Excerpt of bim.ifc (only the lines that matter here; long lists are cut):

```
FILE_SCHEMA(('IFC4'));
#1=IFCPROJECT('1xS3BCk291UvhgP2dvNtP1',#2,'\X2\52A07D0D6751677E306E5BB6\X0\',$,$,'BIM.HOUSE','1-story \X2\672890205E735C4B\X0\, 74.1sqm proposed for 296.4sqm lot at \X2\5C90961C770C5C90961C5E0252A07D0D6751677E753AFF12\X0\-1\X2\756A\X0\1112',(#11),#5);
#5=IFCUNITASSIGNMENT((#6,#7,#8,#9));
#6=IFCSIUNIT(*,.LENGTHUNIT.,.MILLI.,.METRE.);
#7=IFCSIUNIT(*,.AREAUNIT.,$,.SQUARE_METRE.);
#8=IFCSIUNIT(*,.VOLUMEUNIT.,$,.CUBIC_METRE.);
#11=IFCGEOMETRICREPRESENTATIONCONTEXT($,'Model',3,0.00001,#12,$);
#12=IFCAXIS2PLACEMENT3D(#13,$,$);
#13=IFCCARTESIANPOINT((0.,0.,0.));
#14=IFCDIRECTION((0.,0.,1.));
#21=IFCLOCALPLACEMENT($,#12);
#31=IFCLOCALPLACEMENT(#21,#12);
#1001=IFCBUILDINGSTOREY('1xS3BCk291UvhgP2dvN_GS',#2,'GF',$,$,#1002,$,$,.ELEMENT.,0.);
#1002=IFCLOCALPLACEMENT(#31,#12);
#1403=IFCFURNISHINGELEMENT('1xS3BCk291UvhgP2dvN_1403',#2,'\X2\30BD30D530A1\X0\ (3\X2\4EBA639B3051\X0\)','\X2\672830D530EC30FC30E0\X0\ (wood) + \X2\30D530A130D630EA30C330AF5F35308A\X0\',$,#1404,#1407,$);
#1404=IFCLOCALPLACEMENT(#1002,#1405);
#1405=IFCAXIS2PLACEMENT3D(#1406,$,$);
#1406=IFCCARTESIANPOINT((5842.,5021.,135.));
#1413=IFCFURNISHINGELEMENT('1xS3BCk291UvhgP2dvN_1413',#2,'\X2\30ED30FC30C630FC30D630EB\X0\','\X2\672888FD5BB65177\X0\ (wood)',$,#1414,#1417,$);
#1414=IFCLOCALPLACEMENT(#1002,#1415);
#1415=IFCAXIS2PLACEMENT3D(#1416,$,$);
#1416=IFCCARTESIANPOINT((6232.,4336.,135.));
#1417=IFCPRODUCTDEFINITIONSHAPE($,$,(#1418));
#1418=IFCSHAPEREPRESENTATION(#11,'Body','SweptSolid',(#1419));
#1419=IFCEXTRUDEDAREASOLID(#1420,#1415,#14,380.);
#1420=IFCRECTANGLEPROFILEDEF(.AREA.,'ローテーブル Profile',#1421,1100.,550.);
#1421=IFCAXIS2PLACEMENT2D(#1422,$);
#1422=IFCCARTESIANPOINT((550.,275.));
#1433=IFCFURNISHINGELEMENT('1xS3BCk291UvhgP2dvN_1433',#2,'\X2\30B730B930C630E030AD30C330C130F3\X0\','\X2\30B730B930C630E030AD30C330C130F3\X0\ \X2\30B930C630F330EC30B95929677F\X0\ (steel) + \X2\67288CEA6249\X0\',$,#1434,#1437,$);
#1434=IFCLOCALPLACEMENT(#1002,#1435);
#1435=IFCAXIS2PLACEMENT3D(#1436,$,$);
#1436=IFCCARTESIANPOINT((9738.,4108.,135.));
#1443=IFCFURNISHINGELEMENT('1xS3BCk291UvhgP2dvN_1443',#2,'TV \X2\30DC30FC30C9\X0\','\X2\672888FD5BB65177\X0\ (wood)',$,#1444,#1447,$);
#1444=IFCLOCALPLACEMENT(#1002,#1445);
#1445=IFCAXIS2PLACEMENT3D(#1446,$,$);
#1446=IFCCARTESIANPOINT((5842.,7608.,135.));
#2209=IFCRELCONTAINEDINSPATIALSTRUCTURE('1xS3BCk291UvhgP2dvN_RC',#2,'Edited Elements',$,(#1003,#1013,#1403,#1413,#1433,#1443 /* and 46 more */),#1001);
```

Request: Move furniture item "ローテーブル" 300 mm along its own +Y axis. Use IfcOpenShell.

```python
import ifcopenshell
import ifcopenshell.api.geometry
import ifcopenshell.util.placement
import ifcopenshell.util.unit

model = ifcopenshell.open("bim.ifc")
unit_scale = ifcopenshell.util.unit.calculate_unit_scale(model)

item = model.by_id(1413)
matrix = ifcopenshell.util.placement.get_local_placement(item.ObjectPlacement)
matrix[:3, 3] += matrix[:3, 1] * 0.3 / unit_scale
ifcopenshell.api.geometry.edit_object_placement(model, product=item, matrix=matrix, is_si=False)

print(ifcopenshell.util.placement.get_local_placement(item.ObjectPlacement).round(3) + 0.0)

model.write("bim-out.ifc")
```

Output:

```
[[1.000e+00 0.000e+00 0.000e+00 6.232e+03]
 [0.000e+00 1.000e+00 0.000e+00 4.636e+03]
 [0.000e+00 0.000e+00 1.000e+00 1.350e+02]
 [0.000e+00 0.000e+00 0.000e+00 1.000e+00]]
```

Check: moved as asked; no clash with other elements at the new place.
